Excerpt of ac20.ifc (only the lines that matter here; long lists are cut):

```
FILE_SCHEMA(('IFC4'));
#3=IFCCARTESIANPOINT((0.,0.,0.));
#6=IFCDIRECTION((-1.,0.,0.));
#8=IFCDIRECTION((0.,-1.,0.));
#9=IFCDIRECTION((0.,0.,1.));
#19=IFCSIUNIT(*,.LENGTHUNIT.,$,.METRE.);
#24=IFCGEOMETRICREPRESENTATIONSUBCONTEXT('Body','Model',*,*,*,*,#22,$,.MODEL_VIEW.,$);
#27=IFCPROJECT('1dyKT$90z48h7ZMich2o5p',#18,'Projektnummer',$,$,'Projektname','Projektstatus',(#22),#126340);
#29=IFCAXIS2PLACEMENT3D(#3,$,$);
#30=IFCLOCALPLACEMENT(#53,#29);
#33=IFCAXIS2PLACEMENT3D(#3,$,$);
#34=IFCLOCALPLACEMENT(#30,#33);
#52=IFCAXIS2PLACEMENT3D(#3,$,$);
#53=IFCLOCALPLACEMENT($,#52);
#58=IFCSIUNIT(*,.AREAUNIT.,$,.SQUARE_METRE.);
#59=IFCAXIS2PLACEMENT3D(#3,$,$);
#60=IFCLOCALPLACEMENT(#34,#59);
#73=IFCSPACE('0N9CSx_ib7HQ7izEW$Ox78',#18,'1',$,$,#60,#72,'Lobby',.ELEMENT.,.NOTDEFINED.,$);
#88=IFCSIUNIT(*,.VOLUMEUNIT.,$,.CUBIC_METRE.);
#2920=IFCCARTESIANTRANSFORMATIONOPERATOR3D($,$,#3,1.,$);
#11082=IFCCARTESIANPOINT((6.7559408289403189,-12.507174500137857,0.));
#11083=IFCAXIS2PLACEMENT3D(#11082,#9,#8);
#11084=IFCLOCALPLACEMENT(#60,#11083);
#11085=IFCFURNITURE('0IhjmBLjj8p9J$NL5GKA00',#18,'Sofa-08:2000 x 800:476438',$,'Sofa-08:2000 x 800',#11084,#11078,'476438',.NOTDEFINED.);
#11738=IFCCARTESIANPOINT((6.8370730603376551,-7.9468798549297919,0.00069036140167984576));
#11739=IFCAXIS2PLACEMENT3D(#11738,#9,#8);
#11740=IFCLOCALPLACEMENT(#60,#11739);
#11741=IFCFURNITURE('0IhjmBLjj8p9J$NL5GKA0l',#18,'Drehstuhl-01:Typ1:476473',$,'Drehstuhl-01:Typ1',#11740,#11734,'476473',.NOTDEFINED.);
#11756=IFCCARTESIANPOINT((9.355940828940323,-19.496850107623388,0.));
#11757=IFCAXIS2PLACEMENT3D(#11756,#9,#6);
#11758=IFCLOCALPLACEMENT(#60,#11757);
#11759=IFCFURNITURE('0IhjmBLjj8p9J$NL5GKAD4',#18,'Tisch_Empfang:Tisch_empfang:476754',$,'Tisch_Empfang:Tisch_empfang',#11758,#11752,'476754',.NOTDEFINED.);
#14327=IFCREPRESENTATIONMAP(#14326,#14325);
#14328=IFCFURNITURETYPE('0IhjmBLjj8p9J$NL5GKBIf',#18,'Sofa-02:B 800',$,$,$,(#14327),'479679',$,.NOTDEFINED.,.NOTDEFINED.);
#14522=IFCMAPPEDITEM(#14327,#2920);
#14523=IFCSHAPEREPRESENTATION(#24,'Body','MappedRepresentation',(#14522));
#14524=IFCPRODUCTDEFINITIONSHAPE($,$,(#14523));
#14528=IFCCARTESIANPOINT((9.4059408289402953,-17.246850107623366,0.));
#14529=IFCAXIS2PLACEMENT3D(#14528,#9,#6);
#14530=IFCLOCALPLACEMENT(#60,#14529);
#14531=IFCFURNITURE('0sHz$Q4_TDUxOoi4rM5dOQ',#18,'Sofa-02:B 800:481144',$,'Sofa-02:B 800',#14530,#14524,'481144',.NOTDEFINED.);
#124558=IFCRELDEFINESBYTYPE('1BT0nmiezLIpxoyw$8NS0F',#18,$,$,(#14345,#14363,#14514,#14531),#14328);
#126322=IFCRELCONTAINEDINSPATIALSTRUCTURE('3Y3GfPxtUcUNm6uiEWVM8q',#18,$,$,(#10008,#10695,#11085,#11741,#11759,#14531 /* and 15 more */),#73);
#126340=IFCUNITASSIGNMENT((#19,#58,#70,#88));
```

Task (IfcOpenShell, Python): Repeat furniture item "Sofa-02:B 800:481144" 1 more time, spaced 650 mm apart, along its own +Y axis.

```python
import ifcopenshell
import ifcopenshell.api.geometry
import ifcopenshell.api.root
import ifcopenshell.util.element
import ifcopenshell.util.placement
import ifcopenshell.util.unit

model = ifcopenshell.open("ac20.ifc")
unit_scale = ifcopenshell.util.unit.calculate_unit_scale(model)


def reuse_history(source, copy):
    """copy_class also copies each property set's owner history, people and application; keep the originals."""
    for rel in copy.IsDefinedBy:
        if rel.is_a("IfcRelDefinesByProperties") and (history := rel.RelatingPropertyDefinition.OwnerHistory):
            rel.RelatingPropertyDefinition.OwnerHistory = source.OwnerHistory
            ifcopenshell.util.element.remove_deep2(model, history)


source = model.by_guid("0sHz$Q4_TDUxOoi4rM5dOQ")
base = ifcopenshell.util.placement.get_local_placement(source.ObjectPlacement)
step = base[:3, 1] * 0.65 / unit_scale

for i in range(1, 2):
    copy = ifcopenshell.api.root.copy_class(model, product=source)
    copy.Representation = ifcopenshell.util.element.copy_deep(
        model, source.Representation, exclude=["IfcGeometricRepresentationContext", "IfcRepresentationMap"]
    )
    copy.Name = "Sofa-02:B 800"
    copy.Tag = None
    reuse_history(source, copy)
    matrix = base.copy()
    matrix[:3, 3] += i * step
    print("added at", matrix[:3, 3].round(3) + 0.0)
    ifcopenshell.api.geometry.edit_object_placement(model, product=copy, matrix=matrix, is_si=False)

model.write("ac20_edited.ifc")
```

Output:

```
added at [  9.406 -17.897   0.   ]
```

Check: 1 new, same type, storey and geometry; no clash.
